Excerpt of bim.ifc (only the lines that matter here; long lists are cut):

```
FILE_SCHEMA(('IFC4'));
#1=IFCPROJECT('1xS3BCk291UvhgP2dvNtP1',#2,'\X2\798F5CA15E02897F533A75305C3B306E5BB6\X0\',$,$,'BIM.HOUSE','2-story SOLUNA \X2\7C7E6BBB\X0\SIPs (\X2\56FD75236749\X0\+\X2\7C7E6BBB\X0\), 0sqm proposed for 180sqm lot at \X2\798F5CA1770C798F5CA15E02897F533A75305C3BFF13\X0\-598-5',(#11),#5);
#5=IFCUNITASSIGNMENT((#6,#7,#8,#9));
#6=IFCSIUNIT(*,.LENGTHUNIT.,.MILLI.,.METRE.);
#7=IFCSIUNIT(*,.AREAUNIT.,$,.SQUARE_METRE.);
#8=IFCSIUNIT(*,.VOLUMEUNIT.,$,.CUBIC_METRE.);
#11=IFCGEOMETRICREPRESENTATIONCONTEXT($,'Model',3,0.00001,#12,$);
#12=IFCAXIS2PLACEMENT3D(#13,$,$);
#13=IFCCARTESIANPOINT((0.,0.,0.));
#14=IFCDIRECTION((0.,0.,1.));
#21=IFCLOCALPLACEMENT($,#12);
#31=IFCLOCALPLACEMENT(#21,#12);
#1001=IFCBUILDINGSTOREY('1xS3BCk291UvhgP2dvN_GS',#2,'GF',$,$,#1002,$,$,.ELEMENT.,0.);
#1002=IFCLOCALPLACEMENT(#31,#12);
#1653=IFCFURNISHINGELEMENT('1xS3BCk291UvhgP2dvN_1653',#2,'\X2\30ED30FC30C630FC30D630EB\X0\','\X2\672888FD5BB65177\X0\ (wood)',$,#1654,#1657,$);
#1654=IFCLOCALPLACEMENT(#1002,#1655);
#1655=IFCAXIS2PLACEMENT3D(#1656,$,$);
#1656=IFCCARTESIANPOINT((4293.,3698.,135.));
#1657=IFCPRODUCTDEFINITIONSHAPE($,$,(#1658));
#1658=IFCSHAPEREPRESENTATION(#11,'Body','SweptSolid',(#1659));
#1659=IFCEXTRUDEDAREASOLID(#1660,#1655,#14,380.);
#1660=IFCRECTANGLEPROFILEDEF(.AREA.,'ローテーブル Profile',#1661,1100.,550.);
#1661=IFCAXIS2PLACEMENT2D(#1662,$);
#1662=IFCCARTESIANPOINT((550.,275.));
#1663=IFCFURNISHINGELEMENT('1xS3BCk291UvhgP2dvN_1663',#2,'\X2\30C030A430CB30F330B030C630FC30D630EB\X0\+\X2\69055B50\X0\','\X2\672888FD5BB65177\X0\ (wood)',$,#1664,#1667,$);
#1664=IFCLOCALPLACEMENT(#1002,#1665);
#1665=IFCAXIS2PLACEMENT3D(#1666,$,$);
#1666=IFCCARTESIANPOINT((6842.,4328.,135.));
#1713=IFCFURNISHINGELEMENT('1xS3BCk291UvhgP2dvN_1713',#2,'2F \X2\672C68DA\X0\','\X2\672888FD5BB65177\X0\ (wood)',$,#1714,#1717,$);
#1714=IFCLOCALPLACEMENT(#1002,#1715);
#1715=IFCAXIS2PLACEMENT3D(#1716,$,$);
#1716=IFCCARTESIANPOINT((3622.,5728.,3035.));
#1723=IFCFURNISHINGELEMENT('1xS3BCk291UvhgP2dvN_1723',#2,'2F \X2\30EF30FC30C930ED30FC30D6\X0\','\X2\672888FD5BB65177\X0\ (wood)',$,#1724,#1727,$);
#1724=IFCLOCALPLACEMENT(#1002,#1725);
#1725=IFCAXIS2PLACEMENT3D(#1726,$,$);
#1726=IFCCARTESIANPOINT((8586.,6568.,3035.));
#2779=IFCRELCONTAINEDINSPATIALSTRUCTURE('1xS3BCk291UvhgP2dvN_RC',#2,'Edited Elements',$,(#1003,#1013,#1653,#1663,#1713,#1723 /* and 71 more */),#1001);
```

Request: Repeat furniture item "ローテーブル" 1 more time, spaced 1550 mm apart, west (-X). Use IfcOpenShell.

```python
import numpy as np
import ifcopenshell
import ifcopenshell.api.geometry
import ifcopenshell.api.root
import ifcopenshell.util.element
import ifcopenshell.util.placement
import ifcopenshell.util.unit

model = ifcopenshell.open("bim.ifc")
unit_scale = ifcopenshell.util.unit.calculate_unit_scale(model)


def reuse_history(source, copy):
    """copy_class also copies each property set's owner history, people and application; keep the originals."""
    for rel in copy.IsDefinedBy:
        if rel.is_a("IfcRelDefinesByProperties") and (history := rel.RelatingPropertyDefinition.OwnerHistory):
            rel.RelatingPropertyDefinition.OwnerHistory = source.OwnerHistory
            ifcopenshell.util.element.remove_deep2(model, history)


source = model.by_guid("1xS3BCk291UvhgP2dvN_1653")
base = ifcopenshell.util.placement.get_local_placement(source.ObjectPlacement)
step = np.array([-1.0, 0.0, 0.0]) * 1.55 / unit_scale

for i in range(1, 2):
    copy = ifcopenshell.api.root.copy_class(model, product=source)
    copy.Representation = ifcopenshell.util.element.copy_deep(
        model, source.Representation, exclude=["IfcGeometricRepresentationContext", "IfcRepresentationMap"]
    )
    reuse_history(source, copy)
    matrix = base.copy()
    matrix[:3, 3] += i * step
    print("added at", matrix[:3, 3].round(3) + 0.0)
    ifcopenshell.api.geometry.edit_object_placement(model, product=copy, matrix=matrix, is_si=False)

model.write("bim_rev.ifc")
```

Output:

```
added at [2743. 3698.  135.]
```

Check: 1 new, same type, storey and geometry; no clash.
